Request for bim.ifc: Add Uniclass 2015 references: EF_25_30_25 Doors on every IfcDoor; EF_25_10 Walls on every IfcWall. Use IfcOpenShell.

First a look at what the model holds.

```python
import ifcopenshell

model = ifcopenshell.open("bim.ifc")
print(model.schema)
print("classifications:", [c.Name for c in model.by_type("IfcClassification")])
for ifc_class in ("IfcDoor", "IfcRoof", "IfcStair", "IfcWall", "IfcWindow"):
    print(ifc_class, len(model.by_type(ifc_class)))
```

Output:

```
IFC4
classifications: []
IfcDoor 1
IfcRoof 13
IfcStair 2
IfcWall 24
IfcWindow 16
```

```python
import ifcopenshell
import ifcopenshell.api.classification

model = ifcopenshell.open("bim.ifc")

system = ifcopenshell.api.classification.add_classification(model, classification="Uniclass 2015")

codes = {
    "IfcDoor": ("EF_25_30_25", "Doors"),
    "IfcWall": ("EF_25_10", "Walls"),
}
for ifc_class, (code, name) in codes.items():
    products = model.by_type(ifc_class)
    ifcopenshell.api.classification.add_reference(
        model, products=products, classification=system, identification=code, name=name
    )
    print(code, len(products))

model.write("bim_rev.ifc")
```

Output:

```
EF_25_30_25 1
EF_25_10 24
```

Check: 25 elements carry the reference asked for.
